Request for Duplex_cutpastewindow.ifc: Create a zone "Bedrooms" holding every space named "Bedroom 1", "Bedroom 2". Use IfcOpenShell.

First a look at what the model holds.

```python
import ifcopenshell

model = ifcopenshell.open("Duplex_cutpastewindow.ifc")
print(model.schema)
seen = {}
for space in model.by_type("IfcSpace"):
    seen[space.LongName] = seen.get(space.LongName, 0) + 1
for name, count in sorted(seen.items(), key=str):
    print(count, "x", name)
print("zones:", [z.Name for z in model.by_type("IfcZone")][:20])
```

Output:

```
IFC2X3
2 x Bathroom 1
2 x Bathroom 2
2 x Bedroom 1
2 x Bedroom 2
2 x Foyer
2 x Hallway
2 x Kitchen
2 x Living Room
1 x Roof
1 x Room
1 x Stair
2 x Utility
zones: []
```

```python
import ifcopenshell
import ifcopenshell.api.group
import ifcopenshell.api.root

model = ifcopenshell.open("Duplex_cutpastewindow.ifc")

names = {"Bedroom 1", "Bedroom 2"}
spaces = [s for s in model.by_type("IfcSpace") if s.LongName in names]

zone = ifcopenshell.api.root.create_entity(model, ifc_class="IfcZone", name="Bedrooms")
ifcopenshell.api.group.assign_group(model, products=spaces, group=zone)
print(len(spaces), "spaces in", zone.Name)

model.write("Duplex_cutpastewindow_updated.ifc")
```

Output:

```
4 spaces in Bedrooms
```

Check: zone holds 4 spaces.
